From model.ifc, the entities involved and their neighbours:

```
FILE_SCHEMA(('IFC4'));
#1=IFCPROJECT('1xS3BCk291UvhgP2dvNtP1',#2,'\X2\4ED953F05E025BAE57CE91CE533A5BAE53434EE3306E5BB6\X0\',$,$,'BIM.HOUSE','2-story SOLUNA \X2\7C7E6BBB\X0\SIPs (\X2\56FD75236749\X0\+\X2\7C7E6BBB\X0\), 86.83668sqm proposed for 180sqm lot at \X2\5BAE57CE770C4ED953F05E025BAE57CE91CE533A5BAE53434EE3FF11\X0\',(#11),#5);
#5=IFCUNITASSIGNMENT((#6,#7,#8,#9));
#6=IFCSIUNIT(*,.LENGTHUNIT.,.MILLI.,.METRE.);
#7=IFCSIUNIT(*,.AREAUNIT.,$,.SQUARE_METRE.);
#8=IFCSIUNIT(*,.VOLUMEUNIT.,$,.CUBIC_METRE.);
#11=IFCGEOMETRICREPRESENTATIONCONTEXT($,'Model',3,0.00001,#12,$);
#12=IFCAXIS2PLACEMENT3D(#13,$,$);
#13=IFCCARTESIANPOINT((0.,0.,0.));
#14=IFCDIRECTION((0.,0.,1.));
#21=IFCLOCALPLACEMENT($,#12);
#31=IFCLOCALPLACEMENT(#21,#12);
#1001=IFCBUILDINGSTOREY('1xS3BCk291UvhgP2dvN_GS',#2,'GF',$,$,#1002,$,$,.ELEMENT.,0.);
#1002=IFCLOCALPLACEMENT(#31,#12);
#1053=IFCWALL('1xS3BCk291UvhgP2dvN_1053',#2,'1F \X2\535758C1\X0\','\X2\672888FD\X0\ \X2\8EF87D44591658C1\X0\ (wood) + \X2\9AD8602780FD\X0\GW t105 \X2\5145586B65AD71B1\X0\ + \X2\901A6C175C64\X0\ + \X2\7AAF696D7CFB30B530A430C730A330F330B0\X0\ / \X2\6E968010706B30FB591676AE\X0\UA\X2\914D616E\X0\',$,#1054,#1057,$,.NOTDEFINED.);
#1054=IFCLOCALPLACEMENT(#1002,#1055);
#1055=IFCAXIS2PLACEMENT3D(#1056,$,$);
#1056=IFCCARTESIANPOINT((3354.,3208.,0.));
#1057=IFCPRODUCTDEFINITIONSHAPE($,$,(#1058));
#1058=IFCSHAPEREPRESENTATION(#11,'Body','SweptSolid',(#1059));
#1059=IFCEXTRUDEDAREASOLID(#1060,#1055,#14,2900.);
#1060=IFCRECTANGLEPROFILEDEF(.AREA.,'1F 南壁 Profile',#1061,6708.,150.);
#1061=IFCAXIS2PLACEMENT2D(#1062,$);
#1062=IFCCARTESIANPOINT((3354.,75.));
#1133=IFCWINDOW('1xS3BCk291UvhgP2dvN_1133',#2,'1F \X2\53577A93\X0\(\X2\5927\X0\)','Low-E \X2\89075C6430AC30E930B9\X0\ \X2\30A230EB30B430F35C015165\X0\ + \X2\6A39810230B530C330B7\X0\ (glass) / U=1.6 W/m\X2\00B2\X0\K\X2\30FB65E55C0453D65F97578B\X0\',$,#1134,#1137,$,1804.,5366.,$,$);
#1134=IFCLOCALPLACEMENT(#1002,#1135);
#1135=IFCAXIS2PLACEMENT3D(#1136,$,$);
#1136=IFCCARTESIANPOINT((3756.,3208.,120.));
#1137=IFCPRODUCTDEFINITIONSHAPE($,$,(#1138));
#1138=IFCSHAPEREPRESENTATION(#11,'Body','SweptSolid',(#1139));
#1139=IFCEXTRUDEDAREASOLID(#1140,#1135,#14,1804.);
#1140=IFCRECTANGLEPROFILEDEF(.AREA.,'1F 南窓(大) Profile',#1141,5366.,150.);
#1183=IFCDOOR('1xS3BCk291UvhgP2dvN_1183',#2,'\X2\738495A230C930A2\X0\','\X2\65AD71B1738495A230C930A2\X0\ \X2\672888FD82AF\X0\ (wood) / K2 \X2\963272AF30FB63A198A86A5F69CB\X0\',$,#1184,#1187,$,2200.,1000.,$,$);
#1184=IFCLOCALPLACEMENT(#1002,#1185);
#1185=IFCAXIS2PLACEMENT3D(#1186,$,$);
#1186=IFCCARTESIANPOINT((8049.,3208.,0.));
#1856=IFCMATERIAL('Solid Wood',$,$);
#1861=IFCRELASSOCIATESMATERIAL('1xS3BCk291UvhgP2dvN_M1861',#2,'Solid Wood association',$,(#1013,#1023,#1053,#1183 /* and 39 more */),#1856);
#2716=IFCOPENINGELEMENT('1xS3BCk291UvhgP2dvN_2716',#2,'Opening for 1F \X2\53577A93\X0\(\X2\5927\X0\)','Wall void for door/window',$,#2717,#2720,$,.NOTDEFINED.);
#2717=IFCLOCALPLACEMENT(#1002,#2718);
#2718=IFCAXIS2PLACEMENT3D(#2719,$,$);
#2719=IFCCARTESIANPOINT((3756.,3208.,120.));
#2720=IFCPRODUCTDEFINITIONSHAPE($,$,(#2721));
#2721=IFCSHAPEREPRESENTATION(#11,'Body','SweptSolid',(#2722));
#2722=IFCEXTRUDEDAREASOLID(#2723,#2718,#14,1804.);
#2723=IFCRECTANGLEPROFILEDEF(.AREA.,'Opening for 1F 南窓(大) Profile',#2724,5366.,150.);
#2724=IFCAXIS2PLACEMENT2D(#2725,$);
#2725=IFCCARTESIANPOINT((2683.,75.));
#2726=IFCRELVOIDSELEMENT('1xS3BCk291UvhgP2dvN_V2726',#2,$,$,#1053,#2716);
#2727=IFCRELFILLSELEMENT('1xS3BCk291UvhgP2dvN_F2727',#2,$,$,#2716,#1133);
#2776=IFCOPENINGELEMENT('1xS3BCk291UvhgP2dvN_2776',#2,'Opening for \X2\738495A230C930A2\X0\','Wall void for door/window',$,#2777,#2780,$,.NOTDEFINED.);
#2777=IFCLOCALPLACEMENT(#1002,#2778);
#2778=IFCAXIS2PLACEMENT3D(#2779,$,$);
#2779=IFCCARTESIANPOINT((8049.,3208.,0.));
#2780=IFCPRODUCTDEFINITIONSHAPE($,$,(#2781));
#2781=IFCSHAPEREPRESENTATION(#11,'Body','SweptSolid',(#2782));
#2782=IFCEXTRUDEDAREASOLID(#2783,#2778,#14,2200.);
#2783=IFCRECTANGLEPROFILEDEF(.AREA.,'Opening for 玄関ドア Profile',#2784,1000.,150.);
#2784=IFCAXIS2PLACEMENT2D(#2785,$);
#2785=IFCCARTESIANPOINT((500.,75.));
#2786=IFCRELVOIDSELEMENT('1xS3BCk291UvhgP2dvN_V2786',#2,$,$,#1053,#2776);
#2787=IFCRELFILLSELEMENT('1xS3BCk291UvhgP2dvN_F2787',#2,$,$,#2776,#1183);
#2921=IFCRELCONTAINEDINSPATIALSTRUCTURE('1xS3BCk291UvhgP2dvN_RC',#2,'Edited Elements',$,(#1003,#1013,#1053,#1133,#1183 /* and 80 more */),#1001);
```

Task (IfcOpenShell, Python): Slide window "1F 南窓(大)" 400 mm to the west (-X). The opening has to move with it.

```python
import ifcopenshell
import ifcopenshell.api.geometry
import ifcopenshell.util.placement
import ifcopenshell.util.unit

model = ifcopenshell.open("model.ifc")
unit_scale = ifcopenshell.util.unit.calculate_unit_scale(model)

window = model.by_id(1133)
opening = window.FillsVoids[0].RelatingOpeningElement
wall = opening.VoidsElements[0].RelatingBuildingElement

wall_matrix = ifcopenshell.util.placement.get_local_placement(wall.ObjectPlacement)
shift = wall_matrix[:3, 0] * -0.4 / unit_scale
before = ifcopenshell.util.placement.get_local_placement(window.ObjectPlacement)[:3, 3].copy()

# The window is not placed relative to its opening, so move both.
for product in (opening, window):
    matrix = ifcopenshell.util.placement.get_local_placement(product.ObjectPlacement)
    matrix[:3, 3] += shift
    ifcopenshell.api.geometry.edit_object_placement(model, product=product, matrix=matrix, is_si=False)

after = ifcopenshell.util.placement.get_local_placement(window.ObjectPlacement)[:3, 3]
print("window moved by", (after - before).round(3) + 0.0)

model.write("model-out.ifc")
```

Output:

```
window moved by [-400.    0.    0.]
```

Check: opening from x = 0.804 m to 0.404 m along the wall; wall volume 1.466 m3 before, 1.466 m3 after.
